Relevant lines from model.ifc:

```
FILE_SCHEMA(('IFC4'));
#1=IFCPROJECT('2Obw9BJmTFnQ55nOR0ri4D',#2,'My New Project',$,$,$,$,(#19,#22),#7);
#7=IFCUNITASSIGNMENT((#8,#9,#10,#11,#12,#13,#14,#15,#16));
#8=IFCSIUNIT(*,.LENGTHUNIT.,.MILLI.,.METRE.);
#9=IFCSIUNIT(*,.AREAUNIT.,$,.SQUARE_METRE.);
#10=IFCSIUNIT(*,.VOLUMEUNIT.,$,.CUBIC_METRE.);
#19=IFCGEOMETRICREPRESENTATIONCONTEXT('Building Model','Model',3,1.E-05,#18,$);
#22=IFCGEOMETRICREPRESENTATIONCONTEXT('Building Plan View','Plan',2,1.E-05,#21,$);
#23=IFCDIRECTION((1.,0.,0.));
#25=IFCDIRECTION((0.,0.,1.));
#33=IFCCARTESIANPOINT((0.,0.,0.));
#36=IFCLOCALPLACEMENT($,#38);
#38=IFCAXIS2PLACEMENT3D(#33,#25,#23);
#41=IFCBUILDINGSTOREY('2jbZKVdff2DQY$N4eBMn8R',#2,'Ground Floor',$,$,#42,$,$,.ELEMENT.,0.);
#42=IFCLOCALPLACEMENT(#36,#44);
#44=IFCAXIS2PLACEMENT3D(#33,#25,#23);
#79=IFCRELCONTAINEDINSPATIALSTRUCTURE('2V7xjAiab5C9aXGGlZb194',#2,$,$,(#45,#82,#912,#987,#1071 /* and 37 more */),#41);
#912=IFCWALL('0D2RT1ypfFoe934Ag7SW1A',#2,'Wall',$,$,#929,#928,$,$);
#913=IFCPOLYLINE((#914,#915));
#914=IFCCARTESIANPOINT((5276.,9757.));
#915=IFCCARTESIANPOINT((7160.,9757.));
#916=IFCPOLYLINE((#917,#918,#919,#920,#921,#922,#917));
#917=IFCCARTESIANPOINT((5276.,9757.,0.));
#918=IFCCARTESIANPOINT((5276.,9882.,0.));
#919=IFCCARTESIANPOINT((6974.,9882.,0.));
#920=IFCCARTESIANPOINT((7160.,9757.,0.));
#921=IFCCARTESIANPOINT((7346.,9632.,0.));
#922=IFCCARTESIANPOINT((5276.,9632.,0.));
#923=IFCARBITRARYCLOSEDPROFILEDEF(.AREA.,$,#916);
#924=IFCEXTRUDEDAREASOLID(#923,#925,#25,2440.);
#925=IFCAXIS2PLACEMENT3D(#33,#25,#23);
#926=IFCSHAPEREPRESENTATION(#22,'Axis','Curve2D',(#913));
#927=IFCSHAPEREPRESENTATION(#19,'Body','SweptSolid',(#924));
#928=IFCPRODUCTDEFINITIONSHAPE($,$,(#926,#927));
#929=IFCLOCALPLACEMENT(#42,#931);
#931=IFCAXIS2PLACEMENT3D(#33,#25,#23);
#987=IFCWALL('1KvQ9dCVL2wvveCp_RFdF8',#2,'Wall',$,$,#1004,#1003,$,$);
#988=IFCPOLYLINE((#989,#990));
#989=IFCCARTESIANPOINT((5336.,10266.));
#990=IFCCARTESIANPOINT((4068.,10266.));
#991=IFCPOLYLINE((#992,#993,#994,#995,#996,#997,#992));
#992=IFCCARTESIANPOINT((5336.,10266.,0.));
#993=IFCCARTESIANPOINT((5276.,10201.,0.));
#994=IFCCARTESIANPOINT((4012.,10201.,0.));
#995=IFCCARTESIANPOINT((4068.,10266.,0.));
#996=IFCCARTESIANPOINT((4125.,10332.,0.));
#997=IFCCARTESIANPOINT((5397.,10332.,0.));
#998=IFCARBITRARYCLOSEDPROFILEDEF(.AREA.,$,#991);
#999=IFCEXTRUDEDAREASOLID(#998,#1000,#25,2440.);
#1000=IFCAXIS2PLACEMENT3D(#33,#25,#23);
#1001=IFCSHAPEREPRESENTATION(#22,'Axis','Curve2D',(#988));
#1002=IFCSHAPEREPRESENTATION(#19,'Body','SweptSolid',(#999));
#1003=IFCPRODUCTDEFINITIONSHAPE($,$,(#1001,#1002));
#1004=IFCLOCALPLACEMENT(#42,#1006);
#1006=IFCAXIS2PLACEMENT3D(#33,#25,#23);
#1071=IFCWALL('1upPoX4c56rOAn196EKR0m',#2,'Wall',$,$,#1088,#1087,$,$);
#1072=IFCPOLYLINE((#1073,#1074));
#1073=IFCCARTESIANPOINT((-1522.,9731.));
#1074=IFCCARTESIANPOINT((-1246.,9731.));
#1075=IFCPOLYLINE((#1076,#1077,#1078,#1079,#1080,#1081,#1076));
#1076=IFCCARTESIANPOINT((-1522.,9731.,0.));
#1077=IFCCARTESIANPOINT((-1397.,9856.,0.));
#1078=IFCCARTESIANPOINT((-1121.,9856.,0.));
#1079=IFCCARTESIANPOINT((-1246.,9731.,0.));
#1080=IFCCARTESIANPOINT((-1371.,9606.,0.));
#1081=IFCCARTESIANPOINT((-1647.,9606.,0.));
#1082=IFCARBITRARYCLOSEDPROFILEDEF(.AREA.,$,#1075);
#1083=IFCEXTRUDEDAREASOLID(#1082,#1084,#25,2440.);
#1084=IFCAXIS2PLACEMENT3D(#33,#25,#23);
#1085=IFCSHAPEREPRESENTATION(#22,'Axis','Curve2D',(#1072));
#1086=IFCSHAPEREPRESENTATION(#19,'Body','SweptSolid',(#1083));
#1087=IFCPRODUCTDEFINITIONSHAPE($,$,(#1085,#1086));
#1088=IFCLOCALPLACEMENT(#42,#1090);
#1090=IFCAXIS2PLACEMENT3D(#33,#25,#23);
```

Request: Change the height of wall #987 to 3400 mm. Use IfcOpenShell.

```python
import ifcopenshell
import ifcopenshell.geom
import ifcopenshell.util.shape
import ifcopenshell.util.unit

model = ifcopenshell.open("model.ifc")
unit_scale = ifcopenshell.util.unit.calculate_unit_scale(model)
settings = ifcopenshell.geom.settings()


def volume(element):
    """Net volume in cubic metres, openings subtracted."""
    shape = ifcopenshell.geom.create_shape(settings, element)
    return ifcopenshell.util.shape.get_volume(shape.geometry)


wall = model.by_guid("1KvQ9dCVL2wvveCp_RFdF8")
before = volume(wall)

body = next(r for r in wall.Representation.Representations if r.RepresentationIdentifier == "Body")
solid = body.Items[0]
old_height = solid.Depth
solid.Depth = 3.4 / unit_scale
after = volume(wall)

print(f"height {old_height:g} -> {solid.Depth:g}, volume {before:.3f} -> {after:.3f} m3")

model.write("model_v2.ifc")
```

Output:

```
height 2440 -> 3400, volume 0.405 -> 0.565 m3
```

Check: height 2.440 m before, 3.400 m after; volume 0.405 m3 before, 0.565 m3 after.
